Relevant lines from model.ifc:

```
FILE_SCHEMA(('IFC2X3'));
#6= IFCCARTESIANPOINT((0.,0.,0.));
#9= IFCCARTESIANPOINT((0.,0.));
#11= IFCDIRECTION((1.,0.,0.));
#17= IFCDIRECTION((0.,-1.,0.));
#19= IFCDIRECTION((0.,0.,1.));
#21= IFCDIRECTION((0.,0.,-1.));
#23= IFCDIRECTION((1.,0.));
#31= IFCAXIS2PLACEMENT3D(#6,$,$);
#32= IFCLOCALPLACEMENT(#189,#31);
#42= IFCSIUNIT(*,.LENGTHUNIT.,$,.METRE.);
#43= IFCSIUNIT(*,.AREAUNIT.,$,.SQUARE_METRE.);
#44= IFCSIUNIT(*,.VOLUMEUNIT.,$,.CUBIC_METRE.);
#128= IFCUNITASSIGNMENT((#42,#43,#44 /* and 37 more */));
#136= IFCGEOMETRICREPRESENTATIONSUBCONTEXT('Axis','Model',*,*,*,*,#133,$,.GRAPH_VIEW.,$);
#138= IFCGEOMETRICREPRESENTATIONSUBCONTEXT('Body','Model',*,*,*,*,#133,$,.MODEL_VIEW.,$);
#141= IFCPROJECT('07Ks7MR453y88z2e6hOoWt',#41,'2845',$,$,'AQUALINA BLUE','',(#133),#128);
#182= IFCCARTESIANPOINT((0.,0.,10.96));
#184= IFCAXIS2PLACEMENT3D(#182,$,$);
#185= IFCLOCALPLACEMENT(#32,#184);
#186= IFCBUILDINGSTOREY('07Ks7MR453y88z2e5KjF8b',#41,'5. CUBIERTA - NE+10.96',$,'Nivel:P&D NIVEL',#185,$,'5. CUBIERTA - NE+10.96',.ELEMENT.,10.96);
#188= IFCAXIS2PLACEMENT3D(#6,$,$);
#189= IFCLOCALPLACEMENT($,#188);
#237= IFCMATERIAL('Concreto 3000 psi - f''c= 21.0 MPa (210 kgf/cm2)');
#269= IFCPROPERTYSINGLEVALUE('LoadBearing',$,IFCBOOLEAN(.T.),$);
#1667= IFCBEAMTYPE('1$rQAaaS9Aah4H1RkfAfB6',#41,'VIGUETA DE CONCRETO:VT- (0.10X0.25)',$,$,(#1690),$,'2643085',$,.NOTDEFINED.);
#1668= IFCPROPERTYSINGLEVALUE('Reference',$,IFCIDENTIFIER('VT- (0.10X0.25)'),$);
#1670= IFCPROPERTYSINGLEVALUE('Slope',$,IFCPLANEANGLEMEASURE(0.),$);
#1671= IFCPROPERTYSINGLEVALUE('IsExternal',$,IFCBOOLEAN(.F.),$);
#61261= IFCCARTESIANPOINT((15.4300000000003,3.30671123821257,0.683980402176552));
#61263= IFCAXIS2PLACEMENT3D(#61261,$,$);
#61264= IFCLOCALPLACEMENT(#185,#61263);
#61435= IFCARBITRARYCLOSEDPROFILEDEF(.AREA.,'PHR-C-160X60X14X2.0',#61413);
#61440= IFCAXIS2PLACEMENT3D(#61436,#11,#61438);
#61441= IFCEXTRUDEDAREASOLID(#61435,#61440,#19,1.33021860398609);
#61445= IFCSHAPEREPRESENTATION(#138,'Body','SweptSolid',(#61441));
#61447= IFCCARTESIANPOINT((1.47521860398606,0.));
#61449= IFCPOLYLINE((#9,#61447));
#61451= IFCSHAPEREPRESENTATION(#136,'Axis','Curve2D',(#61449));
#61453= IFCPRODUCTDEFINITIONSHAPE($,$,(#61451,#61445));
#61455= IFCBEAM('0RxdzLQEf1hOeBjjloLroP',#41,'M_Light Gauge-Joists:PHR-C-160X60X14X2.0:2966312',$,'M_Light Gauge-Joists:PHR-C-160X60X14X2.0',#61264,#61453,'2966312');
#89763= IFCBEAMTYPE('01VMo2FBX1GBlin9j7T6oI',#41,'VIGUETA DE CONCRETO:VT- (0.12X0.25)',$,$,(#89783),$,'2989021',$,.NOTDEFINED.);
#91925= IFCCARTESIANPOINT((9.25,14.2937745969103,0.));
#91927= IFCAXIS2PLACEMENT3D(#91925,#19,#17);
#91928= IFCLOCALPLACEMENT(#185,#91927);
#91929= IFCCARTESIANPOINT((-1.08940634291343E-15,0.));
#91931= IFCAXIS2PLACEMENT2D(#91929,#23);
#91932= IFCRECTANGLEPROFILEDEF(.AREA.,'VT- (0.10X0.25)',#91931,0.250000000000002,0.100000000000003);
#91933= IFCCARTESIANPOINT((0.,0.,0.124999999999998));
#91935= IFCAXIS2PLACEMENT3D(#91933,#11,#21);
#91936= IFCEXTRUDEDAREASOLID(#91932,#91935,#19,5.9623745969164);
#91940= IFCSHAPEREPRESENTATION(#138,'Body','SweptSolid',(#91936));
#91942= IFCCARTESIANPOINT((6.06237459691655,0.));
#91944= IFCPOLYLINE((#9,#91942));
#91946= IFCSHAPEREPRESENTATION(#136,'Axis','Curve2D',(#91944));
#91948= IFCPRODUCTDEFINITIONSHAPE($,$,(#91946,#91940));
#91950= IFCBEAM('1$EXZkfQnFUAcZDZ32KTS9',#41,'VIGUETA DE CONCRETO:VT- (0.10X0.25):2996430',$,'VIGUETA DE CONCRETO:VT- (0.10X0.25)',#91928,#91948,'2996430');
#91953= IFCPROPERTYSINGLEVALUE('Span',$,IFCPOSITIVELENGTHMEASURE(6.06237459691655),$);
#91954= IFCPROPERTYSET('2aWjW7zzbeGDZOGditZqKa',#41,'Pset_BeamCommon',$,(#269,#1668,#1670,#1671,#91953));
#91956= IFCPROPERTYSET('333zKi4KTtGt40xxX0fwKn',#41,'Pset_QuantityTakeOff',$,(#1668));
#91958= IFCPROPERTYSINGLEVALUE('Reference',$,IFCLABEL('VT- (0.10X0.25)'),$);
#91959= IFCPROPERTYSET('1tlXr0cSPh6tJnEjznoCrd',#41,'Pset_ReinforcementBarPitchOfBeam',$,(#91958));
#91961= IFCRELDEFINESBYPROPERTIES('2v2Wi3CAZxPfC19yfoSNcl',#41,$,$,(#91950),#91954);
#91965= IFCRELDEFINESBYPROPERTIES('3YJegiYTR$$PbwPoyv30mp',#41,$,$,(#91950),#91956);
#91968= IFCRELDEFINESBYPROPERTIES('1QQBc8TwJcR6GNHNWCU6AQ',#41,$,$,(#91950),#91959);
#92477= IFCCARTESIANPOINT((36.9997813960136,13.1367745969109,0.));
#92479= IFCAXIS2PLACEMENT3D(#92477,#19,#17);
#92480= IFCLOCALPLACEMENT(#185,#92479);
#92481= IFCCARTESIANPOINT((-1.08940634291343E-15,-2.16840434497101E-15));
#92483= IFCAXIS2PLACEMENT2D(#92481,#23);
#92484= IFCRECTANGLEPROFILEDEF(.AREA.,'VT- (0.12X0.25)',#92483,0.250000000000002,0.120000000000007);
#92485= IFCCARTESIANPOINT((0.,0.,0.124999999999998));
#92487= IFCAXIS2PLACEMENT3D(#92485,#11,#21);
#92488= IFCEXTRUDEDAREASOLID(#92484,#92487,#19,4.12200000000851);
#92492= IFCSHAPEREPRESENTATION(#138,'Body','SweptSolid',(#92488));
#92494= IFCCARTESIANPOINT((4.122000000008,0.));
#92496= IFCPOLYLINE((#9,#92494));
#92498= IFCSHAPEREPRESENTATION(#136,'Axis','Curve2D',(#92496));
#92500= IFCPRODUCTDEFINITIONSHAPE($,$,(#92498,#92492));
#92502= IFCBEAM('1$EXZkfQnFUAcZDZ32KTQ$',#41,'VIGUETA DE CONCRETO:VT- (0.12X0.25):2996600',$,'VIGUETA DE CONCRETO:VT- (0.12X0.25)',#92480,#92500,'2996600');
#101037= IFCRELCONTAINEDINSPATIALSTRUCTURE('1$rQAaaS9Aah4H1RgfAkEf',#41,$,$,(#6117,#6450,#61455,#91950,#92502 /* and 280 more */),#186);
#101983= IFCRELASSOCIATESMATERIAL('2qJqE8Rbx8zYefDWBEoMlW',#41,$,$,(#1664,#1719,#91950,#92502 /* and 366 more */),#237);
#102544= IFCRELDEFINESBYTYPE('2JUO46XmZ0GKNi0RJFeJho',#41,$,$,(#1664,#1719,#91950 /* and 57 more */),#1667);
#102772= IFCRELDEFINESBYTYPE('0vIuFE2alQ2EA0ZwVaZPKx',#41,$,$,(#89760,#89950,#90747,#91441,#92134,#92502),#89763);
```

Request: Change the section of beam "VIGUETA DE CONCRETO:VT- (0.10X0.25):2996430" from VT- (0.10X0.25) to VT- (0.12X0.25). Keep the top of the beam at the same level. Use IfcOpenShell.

```python
import ifcopenshell
import ifcopenshell.api.pset
import ifcopenshell.api.type
import ifcopenshell.util.element
import ifcopenshell.util.representation

model = ifcopenshell.open("model.ifc")

member = model.by_guid("1$EXZkfQnFUAcZDZ32KTS9")
source = next(p for p in model.by_type("IfcRectangleProfileDef") if p.ProfileName == "VT- (0.12X0.25)")

body = ifcopenshell.util.representation.get_representation(member, "Model", "Body")
solid = body.Items[0]
old_profile = solid.SweptArea

# Copy the section's sizes but keep this member's own profile position.
profile = ifcopenshell.util.element.copy(model, source)
# Profiles are centred, so shift by half the change in depth to hold the top.
shift = (old_profile.XDim - profile.XDim) / 2
x, y = old_profile.Position.Location.Coordinates
up = (-1.0, 0.0)  # upwards, in the solid's own plane
location = model.createIfcCartesianPoint((x + up[0] * shift, y + up[1] * shift))
profile.Position = model.createIfcAxis2Placement2D(location, old_profile.Position.RefDirection)
solid.SweptArea = profile
if not model.get_total_inverses(old_profile):
    ifcopenshell.util.element.remove_deep2(model, old_profile)

new_type = model.by_guid("01VMo2FBX1GBlin9j7T6oI")
ifcopenshell.api.type.assign_type(
    model, related_objects=[member], relating_type=new_type, should_map_representations=False
)
member.Name = member.Name.replace("VT- (0.10X0.25)", "VT- (0.12X0.25)")
member.ObjectType = "VIGUETA DE CONCRETO:VT- (0.12X0.25)"
pset = model.by_id(ifcopenshell.util.element.get_pset(member, "Pset_BeamCommon", should_inherit=False)["id"])
ifcopenshell.api.pset.edit_pset(model, pset=pset, properties={"Reference": "VT- (0.12X0.25)"})
pset = model.by_id(ifcopenshell.util.element.get_pset(member, "Pset_QuantityTakeOff", should_inherit=False)["id"])
ifcopenshell.api.pset.edit_pset(model, pset=pset, properties={"Reference": "VT- (0.12X0.25)"})
pset = model.by_id(ifcopenshell.util.element.get_pset(member, "Pset_ReinforcementBarPitchOfBeam", should_inherit=False)["id"])
ifcopenshell.api.pset.edit_pset(model, pset=pset, properties={"Reference": "VT- (0.12X0.25)"})

print(solid.SweptArea)

model.write("model-out.ifc")
```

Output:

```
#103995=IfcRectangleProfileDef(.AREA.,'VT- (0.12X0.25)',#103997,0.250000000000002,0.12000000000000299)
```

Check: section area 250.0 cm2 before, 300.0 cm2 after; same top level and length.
